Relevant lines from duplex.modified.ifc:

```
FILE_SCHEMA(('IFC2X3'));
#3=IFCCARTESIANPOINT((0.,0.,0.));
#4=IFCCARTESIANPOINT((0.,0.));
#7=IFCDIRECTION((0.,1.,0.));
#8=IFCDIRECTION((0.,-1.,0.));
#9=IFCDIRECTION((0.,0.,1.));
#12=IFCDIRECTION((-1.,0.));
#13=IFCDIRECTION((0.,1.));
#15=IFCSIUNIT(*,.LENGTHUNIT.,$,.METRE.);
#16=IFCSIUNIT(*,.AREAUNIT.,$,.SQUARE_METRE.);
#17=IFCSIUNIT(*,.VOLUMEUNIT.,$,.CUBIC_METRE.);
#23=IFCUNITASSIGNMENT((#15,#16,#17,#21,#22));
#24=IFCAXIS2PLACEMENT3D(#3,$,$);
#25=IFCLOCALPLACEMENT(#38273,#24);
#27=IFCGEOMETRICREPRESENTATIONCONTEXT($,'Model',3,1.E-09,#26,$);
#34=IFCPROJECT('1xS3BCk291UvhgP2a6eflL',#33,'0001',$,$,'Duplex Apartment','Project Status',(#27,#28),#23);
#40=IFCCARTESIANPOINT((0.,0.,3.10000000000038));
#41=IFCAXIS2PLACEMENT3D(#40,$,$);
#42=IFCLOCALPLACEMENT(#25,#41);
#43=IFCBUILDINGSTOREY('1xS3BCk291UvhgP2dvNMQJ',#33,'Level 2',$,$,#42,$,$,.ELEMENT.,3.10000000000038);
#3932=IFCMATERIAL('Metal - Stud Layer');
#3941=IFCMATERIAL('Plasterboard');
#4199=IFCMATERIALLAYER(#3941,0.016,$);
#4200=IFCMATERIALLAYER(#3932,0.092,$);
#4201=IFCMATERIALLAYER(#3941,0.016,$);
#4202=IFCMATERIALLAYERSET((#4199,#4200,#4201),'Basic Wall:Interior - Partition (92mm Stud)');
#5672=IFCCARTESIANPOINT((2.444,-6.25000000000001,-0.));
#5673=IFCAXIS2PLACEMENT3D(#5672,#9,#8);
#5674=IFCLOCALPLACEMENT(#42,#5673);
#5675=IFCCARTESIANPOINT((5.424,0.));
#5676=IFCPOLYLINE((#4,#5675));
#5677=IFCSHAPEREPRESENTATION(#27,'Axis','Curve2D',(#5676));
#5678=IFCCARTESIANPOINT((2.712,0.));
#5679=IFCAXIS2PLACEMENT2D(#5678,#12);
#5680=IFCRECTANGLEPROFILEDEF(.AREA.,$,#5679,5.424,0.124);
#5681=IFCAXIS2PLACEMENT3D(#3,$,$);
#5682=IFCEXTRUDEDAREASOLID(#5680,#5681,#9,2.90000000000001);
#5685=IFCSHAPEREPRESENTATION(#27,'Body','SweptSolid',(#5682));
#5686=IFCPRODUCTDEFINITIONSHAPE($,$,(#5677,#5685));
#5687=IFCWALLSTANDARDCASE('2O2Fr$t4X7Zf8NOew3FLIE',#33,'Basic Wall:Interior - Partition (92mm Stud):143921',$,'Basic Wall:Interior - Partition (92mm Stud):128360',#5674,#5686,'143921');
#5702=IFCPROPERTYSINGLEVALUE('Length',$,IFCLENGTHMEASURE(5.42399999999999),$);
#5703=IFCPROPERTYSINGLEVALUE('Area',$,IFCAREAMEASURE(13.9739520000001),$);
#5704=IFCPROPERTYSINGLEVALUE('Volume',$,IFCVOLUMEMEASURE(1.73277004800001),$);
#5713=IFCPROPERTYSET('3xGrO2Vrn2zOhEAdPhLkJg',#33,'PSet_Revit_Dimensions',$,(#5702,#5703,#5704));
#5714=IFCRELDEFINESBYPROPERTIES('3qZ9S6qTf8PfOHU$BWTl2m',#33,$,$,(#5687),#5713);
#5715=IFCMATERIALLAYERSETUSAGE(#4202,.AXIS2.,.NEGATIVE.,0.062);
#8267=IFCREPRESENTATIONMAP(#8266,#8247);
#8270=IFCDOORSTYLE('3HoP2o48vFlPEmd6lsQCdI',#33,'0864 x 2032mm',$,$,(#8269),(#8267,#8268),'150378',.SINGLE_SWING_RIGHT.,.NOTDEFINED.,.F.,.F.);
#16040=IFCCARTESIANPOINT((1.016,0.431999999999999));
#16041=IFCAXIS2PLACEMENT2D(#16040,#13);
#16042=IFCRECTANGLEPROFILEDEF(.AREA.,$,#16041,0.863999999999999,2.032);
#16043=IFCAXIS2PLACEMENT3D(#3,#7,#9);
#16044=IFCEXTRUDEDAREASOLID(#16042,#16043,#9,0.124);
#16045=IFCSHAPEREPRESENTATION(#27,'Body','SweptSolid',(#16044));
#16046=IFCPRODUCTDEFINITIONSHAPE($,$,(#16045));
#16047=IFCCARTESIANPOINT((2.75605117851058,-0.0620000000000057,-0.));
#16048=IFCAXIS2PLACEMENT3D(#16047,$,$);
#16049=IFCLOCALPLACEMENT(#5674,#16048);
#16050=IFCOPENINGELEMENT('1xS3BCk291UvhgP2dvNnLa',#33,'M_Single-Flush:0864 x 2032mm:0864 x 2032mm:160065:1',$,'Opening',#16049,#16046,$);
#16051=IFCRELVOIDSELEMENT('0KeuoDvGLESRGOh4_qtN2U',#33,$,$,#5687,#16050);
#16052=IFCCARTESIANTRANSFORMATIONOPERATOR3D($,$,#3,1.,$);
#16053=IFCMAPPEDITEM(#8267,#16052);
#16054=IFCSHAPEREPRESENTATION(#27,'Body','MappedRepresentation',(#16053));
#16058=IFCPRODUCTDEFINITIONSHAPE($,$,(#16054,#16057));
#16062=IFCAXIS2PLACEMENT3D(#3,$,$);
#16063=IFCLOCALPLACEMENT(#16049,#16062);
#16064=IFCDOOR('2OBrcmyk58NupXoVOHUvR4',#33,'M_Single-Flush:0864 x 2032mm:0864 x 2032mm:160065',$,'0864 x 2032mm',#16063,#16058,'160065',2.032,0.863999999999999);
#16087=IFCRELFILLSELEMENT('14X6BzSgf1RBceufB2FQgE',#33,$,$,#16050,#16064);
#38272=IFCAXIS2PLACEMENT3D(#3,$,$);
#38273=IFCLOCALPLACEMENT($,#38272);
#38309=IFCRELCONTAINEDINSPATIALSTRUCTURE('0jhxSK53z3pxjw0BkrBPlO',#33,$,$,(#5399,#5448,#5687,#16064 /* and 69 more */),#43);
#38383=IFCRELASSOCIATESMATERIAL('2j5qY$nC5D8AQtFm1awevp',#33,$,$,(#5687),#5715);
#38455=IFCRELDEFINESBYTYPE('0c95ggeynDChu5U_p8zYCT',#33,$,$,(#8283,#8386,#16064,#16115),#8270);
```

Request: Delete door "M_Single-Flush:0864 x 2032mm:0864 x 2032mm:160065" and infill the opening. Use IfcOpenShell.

```python
import ifcopenshell
import ifcopenshell.api.feature
import ifcopenshell.api.pset
import ifcopenshell.api.root
import ifcopenshell.geom
import ifcopenshell.util.element
import ifcopenshell.util.shape
import ifcopenshell.util.unit

model = ifcopenshell.open("duplex.modified.ifc")
area_scale = ifcopenshell.util.unit.calculate_unit_scale(model, "AREAUNIT")
volume_scale = ifcopenshell.util.unit.calculate_unit_scale(model, "VOLUMEUNIT")
settings = ifcopenshell.geom.settings()


def volume(element):
    """Net volume in cubic metres, openings subtracted."""
    shape = ifcopenshell.geom.create_shape(settings, element)
    return ifcopenshell.util.shape.get_volume(shape.geometry)


door = model.by_guid("2OBrcmyk58NupXoVOHUvR4")
opening = door.FillsVoids[0].RelatingOpeningElement
wall = opening.VoidsElements[0].RelatingBuildingElement
before = volume(wall)

ifcopenshell.api.root.remove_product(model, product=door)
ifcopenshell.api.feature.remove_feature(model, feature=opening)

after = volume(wall)
thickness = 0.124  # wall thickness in metres

# Update the wall's stored quantities.
pset = model.by_id(ifcopenshell.util.element.get_pset(wall, "PSet_Revit_Dimensions", should_inherit=False)["id"])
ifcopenshell.api.pset.edit_pset(model, pset=pset, properties={
    "Area": model.create_entity("IfcAreaMeasure", after / thickness / area_scale),
    "Volume": model.create_entity("IfcVolumeMeasure", after / volume_scale),
})

print(f"wall volume {before:.3f} -> {after:.3f} m3")

model.write("duplex.modified-out.ifc")
```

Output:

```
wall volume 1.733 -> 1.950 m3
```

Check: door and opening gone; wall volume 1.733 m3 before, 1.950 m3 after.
